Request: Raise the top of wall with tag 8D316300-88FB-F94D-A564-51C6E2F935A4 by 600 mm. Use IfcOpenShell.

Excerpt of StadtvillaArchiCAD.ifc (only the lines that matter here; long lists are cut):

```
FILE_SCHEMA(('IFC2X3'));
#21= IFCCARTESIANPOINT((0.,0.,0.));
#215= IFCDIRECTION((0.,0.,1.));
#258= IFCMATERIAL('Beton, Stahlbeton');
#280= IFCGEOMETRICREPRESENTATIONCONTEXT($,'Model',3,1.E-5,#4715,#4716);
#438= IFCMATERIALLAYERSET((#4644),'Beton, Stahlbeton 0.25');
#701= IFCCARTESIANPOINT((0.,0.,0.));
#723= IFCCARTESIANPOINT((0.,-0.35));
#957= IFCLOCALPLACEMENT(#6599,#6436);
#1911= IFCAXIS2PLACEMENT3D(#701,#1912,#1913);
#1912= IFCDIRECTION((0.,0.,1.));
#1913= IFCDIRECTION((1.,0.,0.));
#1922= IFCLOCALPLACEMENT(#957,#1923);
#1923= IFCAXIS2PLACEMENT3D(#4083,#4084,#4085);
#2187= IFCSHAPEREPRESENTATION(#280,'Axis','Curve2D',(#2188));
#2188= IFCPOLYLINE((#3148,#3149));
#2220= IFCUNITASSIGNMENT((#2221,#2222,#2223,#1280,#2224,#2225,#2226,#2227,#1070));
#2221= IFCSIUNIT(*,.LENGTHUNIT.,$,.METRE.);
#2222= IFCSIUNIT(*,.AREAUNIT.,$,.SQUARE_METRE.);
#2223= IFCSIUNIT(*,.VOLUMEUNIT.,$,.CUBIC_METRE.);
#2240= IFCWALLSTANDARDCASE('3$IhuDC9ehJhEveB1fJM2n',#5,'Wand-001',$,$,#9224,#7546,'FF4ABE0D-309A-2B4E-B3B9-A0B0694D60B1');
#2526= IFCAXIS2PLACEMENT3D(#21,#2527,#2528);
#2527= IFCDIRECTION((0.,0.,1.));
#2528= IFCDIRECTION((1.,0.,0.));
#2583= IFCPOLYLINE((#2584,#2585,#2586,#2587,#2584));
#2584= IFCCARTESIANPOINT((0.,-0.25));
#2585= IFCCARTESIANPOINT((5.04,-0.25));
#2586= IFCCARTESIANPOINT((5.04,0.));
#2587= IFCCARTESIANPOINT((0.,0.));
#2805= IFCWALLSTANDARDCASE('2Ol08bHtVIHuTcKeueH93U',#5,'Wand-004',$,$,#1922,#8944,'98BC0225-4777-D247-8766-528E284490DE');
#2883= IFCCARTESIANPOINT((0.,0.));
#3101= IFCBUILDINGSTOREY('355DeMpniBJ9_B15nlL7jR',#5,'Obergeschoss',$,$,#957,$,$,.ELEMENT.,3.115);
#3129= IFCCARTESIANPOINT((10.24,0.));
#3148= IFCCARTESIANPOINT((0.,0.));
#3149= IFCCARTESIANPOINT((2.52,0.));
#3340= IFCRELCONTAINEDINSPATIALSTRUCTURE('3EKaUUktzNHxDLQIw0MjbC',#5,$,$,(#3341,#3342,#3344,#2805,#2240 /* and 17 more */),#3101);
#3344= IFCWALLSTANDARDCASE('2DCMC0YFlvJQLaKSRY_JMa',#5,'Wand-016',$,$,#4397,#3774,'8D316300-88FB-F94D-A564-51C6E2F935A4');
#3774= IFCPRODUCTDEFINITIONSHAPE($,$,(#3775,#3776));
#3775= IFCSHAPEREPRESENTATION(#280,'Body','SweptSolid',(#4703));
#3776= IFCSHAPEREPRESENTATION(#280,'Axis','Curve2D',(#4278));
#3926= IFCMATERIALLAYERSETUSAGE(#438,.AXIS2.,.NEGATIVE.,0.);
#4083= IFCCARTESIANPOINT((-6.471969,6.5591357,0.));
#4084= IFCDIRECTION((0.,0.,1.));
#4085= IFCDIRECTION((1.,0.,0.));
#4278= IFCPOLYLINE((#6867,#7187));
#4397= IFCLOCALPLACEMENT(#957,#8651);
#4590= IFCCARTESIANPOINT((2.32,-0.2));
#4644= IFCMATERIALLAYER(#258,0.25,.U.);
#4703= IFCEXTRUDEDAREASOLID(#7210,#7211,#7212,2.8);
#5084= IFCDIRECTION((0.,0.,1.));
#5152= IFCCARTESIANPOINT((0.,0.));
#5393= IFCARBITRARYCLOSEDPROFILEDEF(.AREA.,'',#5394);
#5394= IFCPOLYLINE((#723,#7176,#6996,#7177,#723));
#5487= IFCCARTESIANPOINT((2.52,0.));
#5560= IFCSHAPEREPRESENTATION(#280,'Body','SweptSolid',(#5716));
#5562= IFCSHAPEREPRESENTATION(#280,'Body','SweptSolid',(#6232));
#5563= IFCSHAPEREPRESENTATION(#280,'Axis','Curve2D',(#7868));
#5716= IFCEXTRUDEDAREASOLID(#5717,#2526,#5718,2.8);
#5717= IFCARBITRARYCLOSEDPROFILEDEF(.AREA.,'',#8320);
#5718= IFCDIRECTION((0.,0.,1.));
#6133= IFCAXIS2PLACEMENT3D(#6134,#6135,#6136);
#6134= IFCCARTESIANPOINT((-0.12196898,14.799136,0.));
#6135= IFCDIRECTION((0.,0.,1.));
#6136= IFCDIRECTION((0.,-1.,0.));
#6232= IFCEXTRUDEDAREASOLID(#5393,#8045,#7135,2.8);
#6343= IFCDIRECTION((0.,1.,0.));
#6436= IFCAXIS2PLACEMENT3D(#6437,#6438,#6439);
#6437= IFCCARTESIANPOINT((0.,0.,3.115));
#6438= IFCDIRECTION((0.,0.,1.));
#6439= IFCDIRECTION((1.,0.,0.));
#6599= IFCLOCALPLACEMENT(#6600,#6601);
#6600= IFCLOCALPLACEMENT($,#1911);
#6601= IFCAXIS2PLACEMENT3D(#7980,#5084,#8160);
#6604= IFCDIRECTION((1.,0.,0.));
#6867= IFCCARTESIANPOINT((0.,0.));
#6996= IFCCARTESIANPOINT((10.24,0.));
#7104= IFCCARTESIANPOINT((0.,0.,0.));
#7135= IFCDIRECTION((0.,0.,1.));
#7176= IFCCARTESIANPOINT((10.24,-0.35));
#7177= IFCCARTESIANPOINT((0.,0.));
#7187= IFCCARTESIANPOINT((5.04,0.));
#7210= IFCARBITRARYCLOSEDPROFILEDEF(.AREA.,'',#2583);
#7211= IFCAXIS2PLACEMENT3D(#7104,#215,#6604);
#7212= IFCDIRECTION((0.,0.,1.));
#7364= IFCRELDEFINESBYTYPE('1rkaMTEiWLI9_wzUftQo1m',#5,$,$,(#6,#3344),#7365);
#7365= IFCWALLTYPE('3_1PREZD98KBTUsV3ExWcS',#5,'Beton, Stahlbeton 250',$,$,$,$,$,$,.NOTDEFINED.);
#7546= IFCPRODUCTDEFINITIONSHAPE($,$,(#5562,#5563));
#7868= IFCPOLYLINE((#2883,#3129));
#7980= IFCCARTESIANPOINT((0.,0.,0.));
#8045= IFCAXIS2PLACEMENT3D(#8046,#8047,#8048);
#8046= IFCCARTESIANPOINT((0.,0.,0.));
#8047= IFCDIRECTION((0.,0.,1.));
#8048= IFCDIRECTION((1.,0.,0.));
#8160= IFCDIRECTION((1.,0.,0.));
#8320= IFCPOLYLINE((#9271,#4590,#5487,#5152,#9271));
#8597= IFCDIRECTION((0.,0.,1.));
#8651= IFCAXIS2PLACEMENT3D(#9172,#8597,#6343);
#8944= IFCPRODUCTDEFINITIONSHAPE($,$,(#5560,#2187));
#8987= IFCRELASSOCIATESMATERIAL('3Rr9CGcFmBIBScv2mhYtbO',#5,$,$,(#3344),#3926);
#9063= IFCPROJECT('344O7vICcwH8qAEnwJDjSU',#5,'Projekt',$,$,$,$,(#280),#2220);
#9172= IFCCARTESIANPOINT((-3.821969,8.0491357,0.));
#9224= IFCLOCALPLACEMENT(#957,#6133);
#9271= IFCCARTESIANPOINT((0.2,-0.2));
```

```python
import ifcopenshell
import ifcopenshell.geom
import ifcopenshell.util.shape
import ifcopenshell.util.unit

model = ifcopenshell.open("StadtvillaArchiCAD.ifc")
unit_scale = ifcopenshell.util.unit.calculate_unit_scale(model)
settings = ifcopenshell.geom.settings()


def volume(element):
    """Net volume in cubic metres, openings subtracted."""
    shape = ifcopenshell.geom.create_shape(settings, element)
    return ifcopenshell.util.shape.get_volume(shape.geometry)


wall = model.by_id(3344)
before = volume(wall)

body = next(r for r in wall.Representation.Representations if r.RepresentationIdentifier == "Body")
solid = body.Items[0]
old_height = solid.Depth
solid.Depth += 0.6 / unit_scale
after = volume(wall)

print(f"height {old_height:g} -> {solid.Depth:g}, volume {before:.3f} -> {after:.3f} m3")

model.write("StadtvillaArchiCAD_edited.ifc")
```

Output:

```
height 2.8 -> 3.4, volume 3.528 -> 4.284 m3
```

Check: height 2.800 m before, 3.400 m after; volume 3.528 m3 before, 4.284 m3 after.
